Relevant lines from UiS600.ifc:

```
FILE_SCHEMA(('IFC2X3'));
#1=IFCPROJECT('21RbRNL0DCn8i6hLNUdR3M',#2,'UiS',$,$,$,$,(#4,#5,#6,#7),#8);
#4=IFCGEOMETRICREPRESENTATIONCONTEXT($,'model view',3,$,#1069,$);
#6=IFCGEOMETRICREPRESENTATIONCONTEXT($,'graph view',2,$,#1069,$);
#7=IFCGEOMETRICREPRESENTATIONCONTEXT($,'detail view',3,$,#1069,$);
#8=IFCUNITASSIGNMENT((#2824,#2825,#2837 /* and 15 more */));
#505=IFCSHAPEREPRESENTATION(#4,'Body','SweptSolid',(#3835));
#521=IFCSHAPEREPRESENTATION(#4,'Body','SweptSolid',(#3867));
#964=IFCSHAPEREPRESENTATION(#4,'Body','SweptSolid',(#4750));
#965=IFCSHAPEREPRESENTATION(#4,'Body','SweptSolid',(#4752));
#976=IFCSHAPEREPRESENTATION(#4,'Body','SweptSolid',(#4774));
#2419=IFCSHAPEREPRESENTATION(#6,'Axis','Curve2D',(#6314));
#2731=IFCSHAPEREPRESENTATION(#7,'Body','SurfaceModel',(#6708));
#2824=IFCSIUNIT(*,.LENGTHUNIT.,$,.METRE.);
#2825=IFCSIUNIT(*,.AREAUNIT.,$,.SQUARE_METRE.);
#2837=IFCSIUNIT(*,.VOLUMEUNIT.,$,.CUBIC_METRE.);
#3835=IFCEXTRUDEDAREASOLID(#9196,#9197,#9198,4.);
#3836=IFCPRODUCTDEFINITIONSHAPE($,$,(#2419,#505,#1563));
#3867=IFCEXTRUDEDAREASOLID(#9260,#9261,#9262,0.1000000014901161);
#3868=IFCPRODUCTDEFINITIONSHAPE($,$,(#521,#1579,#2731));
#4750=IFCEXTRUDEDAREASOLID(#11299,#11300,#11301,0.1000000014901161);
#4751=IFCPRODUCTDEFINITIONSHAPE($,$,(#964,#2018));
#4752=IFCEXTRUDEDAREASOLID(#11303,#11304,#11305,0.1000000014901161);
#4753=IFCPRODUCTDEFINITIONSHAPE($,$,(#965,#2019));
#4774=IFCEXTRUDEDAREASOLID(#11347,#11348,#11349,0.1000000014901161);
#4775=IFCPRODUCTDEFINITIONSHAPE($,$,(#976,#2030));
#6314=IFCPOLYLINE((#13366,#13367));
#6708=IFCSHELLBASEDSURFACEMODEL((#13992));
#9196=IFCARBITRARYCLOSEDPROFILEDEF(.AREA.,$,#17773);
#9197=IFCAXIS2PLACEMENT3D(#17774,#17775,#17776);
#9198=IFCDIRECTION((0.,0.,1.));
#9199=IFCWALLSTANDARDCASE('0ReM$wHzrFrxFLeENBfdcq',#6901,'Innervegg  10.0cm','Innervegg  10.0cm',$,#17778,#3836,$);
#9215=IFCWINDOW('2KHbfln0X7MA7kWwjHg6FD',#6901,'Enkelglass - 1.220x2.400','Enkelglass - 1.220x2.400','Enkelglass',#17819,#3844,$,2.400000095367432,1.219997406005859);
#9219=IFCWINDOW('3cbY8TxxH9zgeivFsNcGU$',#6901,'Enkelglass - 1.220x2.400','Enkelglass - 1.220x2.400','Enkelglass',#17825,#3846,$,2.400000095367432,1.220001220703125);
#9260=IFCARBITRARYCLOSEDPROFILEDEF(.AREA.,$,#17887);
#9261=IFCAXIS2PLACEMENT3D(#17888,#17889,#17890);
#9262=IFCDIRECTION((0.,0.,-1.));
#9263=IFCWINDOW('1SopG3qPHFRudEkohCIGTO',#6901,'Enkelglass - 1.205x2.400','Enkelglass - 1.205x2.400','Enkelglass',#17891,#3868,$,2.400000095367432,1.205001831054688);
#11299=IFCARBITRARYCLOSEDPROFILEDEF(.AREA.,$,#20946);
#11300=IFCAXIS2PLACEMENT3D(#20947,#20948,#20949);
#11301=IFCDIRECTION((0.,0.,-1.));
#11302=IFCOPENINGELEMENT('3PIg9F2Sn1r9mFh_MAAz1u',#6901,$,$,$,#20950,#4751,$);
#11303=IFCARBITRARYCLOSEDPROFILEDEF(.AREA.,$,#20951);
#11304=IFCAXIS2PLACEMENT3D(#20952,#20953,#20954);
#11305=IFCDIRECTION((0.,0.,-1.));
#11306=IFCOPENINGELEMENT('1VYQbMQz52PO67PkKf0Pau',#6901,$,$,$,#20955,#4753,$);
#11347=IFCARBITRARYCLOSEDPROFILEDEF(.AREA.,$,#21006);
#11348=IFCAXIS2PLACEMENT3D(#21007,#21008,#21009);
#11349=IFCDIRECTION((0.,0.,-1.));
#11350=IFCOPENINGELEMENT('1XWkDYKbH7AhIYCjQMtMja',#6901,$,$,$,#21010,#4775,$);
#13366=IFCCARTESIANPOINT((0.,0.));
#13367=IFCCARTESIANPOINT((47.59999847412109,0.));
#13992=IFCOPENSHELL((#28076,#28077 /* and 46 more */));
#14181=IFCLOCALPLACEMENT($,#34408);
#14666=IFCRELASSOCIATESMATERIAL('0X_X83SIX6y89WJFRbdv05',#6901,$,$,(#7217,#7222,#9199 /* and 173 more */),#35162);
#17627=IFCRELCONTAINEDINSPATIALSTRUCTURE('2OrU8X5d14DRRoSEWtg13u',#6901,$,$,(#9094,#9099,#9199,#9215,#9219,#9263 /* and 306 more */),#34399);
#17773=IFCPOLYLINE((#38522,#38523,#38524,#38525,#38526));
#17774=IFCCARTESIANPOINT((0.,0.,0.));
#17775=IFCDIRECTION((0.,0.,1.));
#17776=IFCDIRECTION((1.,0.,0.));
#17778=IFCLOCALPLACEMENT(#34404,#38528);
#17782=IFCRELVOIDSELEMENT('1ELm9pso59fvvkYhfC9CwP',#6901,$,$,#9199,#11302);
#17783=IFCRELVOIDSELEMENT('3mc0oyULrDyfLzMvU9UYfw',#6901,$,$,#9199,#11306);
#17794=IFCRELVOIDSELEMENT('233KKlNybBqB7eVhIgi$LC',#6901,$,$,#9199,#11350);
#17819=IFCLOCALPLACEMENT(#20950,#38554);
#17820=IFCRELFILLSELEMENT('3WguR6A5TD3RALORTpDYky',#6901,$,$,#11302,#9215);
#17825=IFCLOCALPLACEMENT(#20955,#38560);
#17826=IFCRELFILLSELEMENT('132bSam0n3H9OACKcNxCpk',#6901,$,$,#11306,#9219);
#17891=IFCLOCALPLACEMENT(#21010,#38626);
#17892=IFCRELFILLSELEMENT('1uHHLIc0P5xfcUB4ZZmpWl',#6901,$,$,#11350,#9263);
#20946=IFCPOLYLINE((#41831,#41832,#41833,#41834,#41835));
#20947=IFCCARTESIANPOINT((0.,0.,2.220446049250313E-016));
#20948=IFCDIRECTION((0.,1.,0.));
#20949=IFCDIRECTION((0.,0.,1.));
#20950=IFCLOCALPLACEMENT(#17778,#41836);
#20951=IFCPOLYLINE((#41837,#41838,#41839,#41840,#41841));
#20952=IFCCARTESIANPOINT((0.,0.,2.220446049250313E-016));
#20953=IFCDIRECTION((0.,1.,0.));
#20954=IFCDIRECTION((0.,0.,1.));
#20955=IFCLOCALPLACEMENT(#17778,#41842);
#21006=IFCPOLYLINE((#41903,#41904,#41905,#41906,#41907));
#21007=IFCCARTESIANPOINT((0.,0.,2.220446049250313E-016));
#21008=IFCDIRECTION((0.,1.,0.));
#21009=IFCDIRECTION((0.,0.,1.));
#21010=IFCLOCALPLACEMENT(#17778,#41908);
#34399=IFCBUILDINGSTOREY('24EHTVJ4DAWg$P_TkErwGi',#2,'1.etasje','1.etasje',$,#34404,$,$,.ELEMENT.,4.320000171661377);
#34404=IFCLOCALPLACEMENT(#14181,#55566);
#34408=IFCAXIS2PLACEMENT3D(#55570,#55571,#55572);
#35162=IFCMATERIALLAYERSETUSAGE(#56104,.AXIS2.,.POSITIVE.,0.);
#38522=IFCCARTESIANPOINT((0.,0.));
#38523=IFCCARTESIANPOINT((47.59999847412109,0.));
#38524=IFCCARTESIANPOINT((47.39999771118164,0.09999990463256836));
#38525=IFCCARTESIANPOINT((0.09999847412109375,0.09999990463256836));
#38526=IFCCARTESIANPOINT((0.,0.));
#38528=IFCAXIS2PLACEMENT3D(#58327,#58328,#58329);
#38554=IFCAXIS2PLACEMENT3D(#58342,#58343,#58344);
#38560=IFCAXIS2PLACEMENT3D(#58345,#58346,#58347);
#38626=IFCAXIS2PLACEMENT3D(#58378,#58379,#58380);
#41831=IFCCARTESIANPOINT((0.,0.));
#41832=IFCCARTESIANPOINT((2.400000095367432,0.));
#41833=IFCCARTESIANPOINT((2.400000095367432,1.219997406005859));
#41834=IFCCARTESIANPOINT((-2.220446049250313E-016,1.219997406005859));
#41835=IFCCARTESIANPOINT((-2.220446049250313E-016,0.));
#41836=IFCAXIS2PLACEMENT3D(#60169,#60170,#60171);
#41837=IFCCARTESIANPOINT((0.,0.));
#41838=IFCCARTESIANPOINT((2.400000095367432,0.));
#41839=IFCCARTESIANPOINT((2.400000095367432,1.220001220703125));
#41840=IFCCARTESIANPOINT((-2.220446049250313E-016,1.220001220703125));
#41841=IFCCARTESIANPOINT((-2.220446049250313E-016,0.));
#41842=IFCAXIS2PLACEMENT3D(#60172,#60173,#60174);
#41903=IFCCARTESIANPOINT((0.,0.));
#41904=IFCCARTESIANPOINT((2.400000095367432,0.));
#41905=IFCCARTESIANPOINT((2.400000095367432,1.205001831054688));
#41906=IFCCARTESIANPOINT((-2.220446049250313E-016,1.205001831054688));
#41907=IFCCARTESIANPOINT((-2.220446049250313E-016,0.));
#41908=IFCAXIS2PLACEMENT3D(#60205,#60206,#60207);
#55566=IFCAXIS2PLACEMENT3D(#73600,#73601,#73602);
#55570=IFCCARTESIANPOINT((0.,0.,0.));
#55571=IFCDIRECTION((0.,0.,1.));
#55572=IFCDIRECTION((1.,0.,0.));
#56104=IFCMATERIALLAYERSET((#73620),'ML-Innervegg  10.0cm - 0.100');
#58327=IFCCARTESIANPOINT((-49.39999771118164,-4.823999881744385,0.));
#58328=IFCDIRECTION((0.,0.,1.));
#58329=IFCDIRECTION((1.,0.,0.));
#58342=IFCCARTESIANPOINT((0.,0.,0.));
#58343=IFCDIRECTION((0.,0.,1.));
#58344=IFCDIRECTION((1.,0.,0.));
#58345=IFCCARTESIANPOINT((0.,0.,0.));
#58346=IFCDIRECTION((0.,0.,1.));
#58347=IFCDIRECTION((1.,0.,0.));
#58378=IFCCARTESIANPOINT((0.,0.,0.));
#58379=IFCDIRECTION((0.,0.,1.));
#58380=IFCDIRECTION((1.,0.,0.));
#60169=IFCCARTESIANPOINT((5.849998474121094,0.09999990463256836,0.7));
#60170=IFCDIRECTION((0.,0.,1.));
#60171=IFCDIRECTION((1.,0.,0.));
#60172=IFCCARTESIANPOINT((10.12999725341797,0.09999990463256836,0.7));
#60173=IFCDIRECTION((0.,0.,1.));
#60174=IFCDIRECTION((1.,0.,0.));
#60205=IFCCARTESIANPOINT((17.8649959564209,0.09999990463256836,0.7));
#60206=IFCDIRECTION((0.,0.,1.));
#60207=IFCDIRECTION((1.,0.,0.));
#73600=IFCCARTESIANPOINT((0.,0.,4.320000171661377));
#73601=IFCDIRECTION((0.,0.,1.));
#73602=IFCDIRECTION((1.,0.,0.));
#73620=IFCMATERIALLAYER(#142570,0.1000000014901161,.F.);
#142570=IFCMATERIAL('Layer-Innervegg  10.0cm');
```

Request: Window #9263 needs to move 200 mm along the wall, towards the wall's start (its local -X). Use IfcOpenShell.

```python
import ifcopenshell
import ifcopenshell.api.geometry
import ifcopenshell.util.placement

model = ifcopenshell.open("UiS600.ifc")

window = model.by_guid("1SopG3qPHFRudEkohCIGTO")
opening = window.FillsVoids[0].RelatingOpeningElement
wall = opening.VoidsElements[0].RelatingBuildingElement

wall_matrix = ifcopenshell.util.placement.get_local_placement(wall.ObjectPlacement)
shift = wall_matrix[:3, 0] * -0.2
before = ifcopenshell.util.placement.get_local_placement(window.ObjectPlacement)[:3, 3].copy()

# The window is placed relative to its opening, so it follows when the opening moves.
matrix = ifcopenshell.util.placement.get_local_placement(opening.ObjectPlacement)
matrix[:3, 3] += shift
ifcopenshell.api.geometry.edit_object_placement(
    model, product=opening, matrix=matrix, is_si=False, should_transform_children=True
)

after = ifcopenshell.util.placement.get_local_placement(window.ObjectPlacement)[:3, 3]
print("window moved by", (after - before).round(3) + 0.0)

model.write("UiS600-out.ifc")
```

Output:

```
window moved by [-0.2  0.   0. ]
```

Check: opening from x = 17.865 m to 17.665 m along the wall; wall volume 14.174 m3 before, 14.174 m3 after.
